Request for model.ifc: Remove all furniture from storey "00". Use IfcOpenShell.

First a look at what the model holds.

```python
import ifcopenshell
import ifcopenshell.util.element

model = ifcopenshell.open("model.ifc")
print(model.schema)
storey = next(s for s in model.by_type("IfcBuildingStorey") if s.Name == "00")
furniture = [e for e in ifcopenshell.util.element.get_decomposition(storey) if e.is_a("IfcFurnishingElement")]
seen = {}
for e in furniture:
    element_type = ifcopenshell.util.element.get_type(e)
    name = element_type.Name if element_type not in (None, e) else None
    seen[name] = seen.get(name, 0) + 1
for name, count in sorted(seen.items(), key=str):
    print(count, "x", name)
```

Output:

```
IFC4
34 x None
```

```python
import ifcopenshell
import ifcopenshell.api.root
import ifcopenshell.util.element

model = ifcopenshell.open("model.ifc")

storey = next(s for s in model.by_type("IfcBuildingStorey") if s.Name == "00")
furniture = [e for e in ifcopenshell.util.element.get_decomposition(storey) if e.is_a("IfcFurnishingElement")]

for e in furniture:
    ifcopenshell.api.root.remove_product(model, product=e)
print(len(furniture), "removed")

model.write("model_v2.ifc")
```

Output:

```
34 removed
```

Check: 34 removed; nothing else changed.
